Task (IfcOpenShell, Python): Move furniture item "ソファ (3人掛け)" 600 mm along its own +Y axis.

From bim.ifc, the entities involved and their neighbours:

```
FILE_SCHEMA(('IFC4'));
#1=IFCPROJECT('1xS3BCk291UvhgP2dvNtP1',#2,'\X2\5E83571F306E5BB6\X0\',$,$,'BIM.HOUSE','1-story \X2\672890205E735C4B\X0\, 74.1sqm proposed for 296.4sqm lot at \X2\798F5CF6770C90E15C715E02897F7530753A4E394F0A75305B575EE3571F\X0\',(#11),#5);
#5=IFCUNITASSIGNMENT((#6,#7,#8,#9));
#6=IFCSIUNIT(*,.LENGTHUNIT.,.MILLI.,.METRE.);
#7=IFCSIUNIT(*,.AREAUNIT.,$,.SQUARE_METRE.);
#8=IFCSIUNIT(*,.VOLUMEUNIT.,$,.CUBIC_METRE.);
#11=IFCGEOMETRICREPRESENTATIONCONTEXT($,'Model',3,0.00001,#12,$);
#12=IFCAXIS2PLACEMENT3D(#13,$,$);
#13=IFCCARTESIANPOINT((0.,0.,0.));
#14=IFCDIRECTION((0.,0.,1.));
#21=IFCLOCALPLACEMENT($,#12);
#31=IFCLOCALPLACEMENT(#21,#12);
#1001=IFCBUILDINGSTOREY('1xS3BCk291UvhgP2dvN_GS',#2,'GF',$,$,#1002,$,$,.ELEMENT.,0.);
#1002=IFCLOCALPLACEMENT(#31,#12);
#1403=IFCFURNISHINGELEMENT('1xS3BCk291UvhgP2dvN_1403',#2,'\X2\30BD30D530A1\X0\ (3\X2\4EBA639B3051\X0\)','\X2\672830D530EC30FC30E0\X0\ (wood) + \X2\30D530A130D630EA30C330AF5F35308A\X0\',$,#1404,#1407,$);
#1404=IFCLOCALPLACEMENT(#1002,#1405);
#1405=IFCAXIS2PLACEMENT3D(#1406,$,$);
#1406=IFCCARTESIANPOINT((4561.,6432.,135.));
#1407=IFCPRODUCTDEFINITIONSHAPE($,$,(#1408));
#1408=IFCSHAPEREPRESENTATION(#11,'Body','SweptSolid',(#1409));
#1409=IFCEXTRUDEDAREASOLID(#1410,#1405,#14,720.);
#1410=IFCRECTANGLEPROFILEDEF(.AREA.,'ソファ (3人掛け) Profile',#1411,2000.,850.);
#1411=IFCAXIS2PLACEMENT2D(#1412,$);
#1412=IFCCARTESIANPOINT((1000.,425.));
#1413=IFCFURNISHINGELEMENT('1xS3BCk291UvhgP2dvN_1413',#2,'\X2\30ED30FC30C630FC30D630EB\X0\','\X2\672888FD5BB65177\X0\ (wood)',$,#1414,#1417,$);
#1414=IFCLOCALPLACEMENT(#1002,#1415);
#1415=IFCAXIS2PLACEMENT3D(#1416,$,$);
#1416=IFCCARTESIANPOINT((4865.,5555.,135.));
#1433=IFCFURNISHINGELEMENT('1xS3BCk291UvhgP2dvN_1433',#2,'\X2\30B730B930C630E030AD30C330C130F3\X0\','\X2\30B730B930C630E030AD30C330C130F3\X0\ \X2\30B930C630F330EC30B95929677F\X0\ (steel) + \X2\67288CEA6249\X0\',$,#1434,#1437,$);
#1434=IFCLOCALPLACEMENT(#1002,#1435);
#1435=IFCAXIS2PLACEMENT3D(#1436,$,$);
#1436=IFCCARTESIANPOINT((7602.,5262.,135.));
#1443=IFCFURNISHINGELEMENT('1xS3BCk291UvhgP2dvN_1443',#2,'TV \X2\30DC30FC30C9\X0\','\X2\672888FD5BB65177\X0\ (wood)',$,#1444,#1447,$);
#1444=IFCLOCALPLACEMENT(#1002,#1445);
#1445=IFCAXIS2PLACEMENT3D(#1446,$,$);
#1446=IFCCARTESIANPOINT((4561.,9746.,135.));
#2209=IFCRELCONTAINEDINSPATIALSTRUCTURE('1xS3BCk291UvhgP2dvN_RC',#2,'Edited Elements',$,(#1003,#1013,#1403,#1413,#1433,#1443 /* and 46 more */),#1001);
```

```python
import ifcopenshell
import ifcopenshell.api.geometry
import ifcopenshell.util.placement
import ifcopenshell.util.unit

model = ifcopenshell.open("bim.ifc")
unit_scale = ifcopenshell.util.unit.calculate_unit_scale(model)

item = model.by_guid("1xS3BCk291UvhgP2dvN_1403")
matrix = ifcopenshell.util.placement.get_local_placement(item.ObjectPlacement)
matrix[:3, 3] += matrix[:3, 1] * 0.6 / unit_scale
ifcopenshell.api.geometry.edit_object_placement(model, product=item, matrix=matrix, is_si=False)

print(ifcopenshell.util.placement.get_local_placement(item.ObjectPlacement).round(3) + 0.0)

model.write("bim_edited.ifc")
```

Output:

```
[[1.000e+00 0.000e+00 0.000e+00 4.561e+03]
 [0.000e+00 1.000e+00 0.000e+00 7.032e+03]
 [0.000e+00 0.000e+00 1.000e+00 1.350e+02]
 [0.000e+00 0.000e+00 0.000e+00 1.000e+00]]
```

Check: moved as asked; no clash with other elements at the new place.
